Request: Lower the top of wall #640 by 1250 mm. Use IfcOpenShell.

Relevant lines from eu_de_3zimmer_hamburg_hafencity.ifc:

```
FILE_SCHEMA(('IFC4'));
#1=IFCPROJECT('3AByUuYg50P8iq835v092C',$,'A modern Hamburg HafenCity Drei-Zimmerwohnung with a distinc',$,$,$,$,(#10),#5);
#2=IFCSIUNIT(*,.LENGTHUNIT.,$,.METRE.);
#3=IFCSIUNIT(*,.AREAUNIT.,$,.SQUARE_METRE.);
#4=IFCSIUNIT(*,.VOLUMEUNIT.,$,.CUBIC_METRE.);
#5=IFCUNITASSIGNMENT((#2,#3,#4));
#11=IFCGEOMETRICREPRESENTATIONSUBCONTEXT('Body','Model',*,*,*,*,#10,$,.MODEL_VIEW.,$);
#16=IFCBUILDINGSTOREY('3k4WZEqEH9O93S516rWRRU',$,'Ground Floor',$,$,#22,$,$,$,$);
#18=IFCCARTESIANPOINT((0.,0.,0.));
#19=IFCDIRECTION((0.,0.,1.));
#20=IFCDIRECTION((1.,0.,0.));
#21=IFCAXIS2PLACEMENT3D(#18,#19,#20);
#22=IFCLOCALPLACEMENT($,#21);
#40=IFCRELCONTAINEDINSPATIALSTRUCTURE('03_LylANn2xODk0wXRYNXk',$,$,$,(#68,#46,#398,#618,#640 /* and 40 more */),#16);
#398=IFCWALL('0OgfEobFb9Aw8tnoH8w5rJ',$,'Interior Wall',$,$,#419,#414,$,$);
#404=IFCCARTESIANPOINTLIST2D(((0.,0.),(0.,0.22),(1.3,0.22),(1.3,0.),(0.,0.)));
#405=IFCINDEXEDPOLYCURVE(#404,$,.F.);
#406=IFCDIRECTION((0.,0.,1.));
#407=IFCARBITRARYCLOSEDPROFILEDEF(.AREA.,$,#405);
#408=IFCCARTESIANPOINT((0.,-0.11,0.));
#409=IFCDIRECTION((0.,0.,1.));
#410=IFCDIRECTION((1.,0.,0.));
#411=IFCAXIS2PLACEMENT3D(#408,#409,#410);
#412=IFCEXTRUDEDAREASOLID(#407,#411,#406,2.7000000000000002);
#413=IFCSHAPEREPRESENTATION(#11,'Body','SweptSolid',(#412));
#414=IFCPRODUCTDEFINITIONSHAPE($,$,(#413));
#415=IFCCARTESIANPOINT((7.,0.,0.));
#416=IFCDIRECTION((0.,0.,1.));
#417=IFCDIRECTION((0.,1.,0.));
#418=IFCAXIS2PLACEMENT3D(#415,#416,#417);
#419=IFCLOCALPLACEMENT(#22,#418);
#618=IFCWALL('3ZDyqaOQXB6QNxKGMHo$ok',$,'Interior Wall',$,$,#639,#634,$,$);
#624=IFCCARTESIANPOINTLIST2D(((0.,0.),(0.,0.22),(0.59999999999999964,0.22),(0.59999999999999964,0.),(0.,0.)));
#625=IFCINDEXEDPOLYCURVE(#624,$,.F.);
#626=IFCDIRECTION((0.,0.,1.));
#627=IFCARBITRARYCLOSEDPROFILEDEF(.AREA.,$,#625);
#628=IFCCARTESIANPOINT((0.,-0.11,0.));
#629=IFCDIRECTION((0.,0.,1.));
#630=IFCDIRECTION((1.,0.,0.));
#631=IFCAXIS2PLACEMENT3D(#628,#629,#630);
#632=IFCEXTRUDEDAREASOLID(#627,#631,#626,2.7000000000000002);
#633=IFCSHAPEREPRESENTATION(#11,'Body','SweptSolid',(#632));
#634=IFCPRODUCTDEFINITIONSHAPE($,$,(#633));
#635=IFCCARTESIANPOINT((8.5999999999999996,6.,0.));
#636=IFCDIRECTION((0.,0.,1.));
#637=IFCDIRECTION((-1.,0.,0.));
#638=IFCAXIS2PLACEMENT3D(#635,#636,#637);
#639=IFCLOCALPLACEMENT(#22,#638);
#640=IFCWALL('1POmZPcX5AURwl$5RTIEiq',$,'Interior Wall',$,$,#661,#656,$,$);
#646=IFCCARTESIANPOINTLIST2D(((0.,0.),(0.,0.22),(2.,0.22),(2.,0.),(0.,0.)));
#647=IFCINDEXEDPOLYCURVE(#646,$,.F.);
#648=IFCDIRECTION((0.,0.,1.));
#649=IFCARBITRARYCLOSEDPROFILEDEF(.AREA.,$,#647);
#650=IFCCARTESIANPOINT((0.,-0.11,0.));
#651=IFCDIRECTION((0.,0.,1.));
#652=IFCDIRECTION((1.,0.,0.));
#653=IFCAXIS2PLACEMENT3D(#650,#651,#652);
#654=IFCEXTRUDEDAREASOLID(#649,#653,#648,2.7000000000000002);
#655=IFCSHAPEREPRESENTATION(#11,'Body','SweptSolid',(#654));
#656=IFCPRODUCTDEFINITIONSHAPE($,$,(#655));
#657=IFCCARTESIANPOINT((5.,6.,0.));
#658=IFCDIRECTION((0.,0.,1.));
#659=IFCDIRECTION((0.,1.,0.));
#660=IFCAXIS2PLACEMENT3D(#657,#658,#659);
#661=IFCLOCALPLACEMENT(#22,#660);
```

```python
import ifcopenshell
import ifcopenshell.geom
import ifcopenshell.util.representation
import ifcopenshell.util.shape
import ifcopenshell.util.unit

model = ifcopenshell.open("eu_de_3zimmer_hamburg_hafencity.ifc")
unit_scale = ifcopenshell.util.unit.calculate_unit_scale(model)
settings = ifcopenshell.geom.settings()


def volume(element):
    """Net volume in cubic metres, openings subtracted."""
    shape = ifcopenshell.geom.create_shape(settings, element)
    return ifcopenshell.util.shape.get_volume(shape.geometry)


wall = model.by_guid("1POmZPcX5AURwl$5RTIEiq")
before = volume(wall)

body = ifcopenshell.util.representation.get_representation(wall, "Model", "Body")
solid = body.Items[0]
old_height = solid.Depth
solid.Depth -= 1.25 / unit_scale
after = volume(wall)

print(f"height {old_height:g} -> {solid.Depth:g}, volume {before:.3f} -> {after:.3f} m3")

model.write("eu_de_3zimmer_hamburg_hafencity_rev.ifc")
```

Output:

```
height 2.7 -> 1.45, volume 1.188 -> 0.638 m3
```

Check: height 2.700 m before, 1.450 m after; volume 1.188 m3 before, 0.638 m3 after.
